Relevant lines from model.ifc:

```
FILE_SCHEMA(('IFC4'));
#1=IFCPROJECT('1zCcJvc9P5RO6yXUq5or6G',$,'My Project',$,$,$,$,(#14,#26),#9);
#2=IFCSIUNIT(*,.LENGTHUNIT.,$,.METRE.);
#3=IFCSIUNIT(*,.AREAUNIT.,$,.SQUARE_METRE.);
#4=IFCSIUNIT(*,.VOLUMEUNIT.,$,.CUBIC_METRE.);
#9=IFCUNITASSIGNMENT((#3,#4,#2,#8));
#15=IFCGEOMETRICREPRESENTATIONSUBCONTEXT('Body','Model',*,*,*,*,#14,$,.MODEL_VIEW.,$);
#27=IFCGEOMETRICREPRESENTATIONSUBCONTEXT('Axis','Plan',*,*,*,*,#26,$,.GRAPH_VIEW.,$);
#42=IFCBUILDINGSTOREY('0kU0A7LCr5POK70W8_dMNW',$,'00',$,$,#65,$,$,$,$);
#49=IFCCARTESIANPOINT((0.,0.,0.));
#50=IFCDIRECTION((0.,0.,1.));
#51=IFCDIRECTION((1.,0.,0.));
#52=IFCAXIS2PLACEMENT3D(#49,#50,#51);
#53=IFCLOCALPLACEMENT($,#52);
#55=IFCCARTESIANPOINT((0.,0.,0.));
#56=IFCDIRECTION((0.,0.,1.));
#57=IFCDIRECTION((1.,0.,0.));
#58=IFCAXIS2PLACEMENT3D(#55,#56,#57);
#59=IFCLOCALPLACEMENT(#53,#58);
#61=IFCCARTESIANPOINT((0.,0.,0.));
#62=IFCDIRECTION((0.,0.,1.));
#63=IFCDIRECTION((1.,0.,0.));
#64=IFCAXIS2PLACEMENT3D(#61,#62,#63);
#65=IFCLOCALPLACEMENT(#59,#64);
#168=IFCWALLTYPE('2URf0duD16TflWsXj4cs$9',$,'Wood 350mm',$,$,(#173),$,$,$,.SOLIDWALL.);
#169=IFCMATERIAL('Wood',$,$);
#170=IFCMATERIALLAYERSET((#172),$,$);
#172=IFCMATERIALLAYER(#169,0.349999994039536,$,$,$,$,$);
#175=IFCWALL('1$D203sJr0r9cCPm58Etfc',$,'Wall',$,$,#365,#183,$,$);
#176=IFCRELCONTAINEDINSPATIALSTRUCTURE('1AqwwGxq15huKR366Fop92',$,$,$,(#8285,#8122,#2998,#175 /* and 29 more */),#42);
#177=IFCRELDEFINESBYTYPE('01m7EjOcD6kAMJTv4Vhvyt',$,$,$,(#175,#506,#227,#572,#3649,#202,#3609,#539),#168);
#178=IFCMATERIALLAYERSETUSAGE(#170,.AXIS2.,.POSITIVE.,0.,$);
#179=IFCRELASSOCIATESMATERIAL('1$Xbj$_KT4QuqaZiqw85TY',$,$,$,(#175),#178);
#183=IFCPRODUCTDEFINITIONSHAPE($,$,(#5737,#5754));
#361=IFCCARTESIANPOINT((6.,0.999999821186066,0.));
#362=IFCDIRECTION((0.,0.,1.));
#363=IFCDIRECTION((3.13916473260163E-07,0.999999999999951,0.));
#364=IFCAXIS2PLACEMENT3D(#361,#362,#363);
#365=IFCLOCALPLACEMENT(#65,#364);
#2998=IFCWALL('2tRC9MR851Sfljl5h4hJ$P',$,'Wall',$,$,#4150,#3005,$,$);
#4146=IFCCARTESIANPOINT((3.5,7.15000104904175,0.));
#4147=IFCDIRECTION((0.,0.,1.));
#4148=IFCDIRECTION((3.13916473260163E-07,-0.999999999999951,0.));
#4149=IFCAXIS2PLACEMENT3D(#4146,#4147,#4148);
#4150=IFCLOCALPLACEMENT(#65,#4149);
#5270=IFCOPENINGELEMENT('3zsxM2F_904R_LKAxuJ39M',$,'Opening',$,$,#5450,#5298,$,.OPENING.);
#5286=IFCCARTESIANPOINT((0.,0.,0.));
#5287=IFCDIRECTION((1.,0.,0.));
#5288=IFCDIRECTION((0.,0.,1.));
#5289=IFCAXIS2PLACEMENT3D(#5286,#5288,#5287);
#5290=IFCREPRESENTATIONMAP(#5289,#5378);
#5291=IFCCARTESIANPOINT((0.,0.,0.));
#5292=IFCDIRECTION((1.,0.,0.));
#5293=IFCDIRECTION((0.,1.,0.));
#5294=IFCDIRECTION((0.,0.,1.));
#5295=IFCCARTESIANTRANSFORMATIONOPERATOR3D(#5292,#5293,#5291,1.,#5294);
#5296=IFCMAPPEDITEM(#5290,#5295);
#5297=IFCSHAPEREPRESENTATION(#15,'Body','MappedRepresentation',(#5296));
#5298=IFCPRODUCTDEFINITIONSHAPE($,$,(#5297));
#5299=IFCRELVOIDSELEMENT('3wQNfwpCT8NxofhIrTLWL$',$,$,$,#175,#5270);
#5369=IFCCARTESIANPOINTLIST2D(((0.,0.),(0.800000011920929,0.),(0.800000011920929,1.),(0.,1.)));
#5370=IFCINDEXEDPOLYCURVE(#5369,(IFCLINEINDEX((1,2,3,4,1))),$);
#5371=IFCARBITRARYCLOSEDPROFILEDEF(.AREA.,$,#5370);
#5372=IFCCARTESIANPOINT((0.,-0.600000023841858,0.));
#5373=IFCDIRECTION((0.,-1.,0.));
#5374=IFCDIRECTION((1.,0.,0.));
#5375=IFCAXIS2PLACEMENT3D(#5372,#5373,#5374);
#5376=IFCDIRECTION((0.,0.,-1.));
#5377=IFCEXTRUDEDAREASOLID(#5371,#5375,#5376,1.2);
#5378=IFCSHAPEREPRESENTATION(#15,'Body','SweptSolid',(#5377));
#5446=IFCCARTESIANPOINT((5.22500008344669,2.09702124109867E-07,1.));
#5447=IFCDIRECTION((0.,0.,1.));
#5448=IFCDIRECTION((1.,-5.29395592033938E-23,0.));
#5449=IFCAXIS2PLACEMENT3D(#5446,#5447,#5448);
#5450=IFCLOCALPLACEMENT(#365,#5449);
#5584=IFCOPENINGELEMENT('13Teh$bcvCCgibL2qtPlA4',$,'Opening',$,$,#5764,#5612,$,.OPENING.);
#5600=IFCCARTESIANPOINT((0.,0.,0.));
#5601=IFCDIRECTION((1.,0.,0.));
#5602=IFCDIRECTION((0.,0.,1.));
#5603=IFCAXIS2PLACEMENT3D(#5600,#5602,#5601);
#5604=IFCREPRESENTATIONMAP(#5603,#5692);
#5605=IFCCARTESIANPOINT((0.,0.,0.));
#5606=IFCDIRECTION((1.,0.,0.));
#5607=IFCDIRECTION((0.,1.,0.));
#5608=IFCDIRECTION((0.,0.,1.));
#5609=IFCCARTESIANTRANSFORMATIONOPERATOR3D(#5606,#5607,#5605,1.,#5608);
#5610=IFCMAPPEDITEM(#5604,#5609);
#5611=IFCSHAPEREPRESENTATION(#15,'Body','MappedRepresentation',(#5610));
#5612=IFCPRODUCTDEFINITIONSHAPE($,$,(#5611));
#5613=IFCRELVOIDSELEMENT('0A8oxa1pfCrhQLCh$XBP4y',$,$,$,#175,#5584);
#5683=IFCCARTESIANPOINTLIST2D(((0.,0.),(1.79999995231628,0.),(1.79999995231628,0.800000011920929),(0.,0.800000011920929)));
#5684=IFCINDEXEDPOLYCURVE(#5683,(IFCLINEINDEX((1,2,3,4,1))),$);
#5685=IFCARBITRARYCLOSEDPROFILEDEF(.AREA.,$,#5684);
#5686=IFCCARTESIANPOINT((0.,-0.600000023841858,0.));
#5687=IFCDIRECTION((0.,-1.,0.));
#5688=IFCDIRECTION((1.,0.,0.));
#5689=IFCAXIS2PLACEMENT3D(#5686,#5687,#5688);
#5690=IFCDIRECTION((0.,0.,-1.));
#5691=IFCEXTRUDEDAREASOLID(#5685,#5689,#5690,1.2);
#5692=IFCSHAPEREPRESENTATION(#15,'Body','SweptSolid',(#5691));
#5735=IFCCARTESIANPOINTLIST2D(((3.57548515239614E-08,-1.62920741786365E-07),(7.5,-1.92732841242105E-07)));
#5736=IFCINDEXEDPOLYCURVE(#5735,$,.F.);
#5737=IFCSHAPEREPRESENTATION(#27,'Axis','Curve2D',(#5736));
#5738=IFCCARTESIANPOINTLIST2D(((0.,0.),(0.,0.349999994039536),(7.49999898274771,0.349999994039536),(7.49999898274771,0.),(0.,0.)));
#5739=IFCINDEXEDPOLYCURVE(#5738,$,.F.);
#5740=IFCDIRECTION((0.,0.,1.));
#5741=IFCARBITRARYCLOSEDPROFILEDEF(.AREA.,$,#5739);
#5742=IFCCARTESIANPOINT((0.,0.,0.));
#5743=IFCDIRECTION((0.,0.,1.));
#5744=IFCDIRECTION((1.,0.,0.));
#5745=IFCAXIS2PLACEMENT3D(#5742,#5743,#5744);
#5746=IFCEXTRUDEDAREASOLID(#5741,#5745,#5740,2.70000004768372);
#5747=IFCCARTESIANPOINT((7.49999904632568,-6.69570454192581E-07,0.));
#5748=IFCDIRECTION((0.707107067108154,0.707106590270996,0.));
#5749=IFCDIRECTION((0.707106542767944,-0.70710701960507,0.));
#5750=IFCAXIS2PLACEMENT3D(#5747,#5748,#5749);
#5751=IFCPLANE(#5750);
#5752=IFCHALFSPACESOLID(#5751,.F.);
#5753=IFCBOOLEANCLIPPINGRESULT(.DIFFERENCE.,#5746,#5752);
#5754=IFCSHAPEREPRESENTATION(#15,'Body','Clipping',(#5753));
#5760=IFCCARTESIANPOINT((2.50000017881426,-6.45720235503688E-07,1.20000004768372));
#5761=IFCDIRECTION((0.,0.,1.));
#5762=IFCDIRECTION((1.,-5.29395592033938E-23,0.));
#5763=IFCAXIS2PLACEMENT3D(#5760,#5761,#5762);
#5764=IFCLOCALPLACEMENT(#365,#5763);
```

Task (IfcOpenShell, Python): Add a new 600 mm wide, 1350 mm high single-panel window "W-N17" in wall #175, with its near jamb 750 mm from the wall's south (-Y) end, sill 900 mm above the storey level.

```python
import numpy as np
import ifcopenshell
import ifcopenshell.api.feature
import ifcopenshell.api.geometry
import ifcopenshell.api.root
import ifcopenshell.api.spatial
import ifcopenshell.geom
import ifcopenshell.util.element
import ifcopenshell.util.placement
import ifcopenshell.util.representation
import ifcopenshell.util.shape
import ifcopenshell.util.unit

model = ifcopenshell.open("model.ifc")
unit_scale = ifcopenshell.util.unit.calculate_unit_scale(model)
settings = ifcopenshell.geom.settings()


def volume(element):
    """Net volume in cubic metres, openings subtracted."""
    shape = ifcopenshell.geom.create_shape(settings, element)
    return ifcopenshell.util.shape.get_volume(shape.geometry)


wall = model.by_id(175)
storey = ifcopenshell.util.element.get_container(wall, ifc_class="IfcBuildingStorey")
context = ifcopenshell.util.representation.get_context(model, "Model", "Body", "MODEL_VIEW")
before = volume(wall)

width, height, from_end, sill = 0.6, 1.35, 0.75, 0.9  # metres

# The wall runs along its own X axis, and the end named is its -X end.
wall_shape = ifcopenshell.geom.create_shape(settings, wall)
x, y, z = ifcopenshell.util.shape.get_vertices(wall_shape.geometry).T
start = x.min() + from_end
face, thickness = float(y.min()), float(y.max() - y.min())
wall_matrix = ifcopenshell.util.placement.get_local_placement(wall.ObjectPlacement)
level = ifcopenshell.util.placement.get_local_placement(storey.ObjectPlacement)[2, 3]


def in_wall(x, y):
    """Placement at x, y metres in the wall's axes, at sill height."""
    matrix = wall_matrix.copy()
    matrix[:, 3] = wall_matrix @ np.array([x / unit_scale, y / unit_scale, 0.0, 1.0])
    matrix[2, 3] = level + sill / unit_scale
    return matrix


# Opening: a box that overshoots both wall faces by 50 mm.
opening = ifcopenshell.api.root.create_entity(model, ifc_class="IfcOpeningElement", predefined_type="OPENING")
box = ifcopenshell.api.geometry.add_wall_representation(
    model, context=context, length=width, height=height, thickness=thickness + 0.1
)
ifcopenshell.api.geometry.assign_representation(model, product=opening, representation=box)
ifcopenshell.api.geometry.edit_object_placement(model, product=opening, matrix=in_wall(start, face - 0.05), is_si=False)
ifcopenshell.api.feature.add_feature(model, feature=opening, element=wall)

window = ifcopenshell.api.root.create_entity(model, ifc_class="IfcWindow", name="W-N17", predefined_type="WINDOW")
window.OverallWidth, window.OverallHeight = width / unit_scale, height / unit_scale
window.PartitioningType = "SINGLE_PANEL"
body = ifcopenshell.api.geometry.add_window_representation(
    model,
    context=context,
    overall_width=window.OverallWidth,
    overall_height=window.OverallHeight,
    partition_type="SINGLE_PANEL",
)
ifcopenshell.api.geometry.assign_representation(model, product=window, representation=body)
ifcopenshell.api.spatial.assign_container(model, products=[window], relating_structure=storey)
ifcopenshell.api.feature.add_filling(model, opening=opening, element=window)

# Centre the window in the wall's thickness.
ifcopenshell.api.geometry.edit_object_placement(model, product=window, matrix=in_wall(start, face), is_si=False)
window_shape = ifcopenshell.geom.create_shape(settings, window)
depth = ifcopenshell.util.shape.get_vertices(window_shape.geometry)[:, 1]
offset = face + thickness / 2 - (depth.min() + depth.max()) / 2
ifcopenshell.api.geometry.edit_object_placement(model, product=window, matrix=in_wall(start, offset), is_si=False)

after = volume(wall)

print(f"wall volume {before:.3f} -> {after:.3f} m3")

model.write("model_v2.ifc")
```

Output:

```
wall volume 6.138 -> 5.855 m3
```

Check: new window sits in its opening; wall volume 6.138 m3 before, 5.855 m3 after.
